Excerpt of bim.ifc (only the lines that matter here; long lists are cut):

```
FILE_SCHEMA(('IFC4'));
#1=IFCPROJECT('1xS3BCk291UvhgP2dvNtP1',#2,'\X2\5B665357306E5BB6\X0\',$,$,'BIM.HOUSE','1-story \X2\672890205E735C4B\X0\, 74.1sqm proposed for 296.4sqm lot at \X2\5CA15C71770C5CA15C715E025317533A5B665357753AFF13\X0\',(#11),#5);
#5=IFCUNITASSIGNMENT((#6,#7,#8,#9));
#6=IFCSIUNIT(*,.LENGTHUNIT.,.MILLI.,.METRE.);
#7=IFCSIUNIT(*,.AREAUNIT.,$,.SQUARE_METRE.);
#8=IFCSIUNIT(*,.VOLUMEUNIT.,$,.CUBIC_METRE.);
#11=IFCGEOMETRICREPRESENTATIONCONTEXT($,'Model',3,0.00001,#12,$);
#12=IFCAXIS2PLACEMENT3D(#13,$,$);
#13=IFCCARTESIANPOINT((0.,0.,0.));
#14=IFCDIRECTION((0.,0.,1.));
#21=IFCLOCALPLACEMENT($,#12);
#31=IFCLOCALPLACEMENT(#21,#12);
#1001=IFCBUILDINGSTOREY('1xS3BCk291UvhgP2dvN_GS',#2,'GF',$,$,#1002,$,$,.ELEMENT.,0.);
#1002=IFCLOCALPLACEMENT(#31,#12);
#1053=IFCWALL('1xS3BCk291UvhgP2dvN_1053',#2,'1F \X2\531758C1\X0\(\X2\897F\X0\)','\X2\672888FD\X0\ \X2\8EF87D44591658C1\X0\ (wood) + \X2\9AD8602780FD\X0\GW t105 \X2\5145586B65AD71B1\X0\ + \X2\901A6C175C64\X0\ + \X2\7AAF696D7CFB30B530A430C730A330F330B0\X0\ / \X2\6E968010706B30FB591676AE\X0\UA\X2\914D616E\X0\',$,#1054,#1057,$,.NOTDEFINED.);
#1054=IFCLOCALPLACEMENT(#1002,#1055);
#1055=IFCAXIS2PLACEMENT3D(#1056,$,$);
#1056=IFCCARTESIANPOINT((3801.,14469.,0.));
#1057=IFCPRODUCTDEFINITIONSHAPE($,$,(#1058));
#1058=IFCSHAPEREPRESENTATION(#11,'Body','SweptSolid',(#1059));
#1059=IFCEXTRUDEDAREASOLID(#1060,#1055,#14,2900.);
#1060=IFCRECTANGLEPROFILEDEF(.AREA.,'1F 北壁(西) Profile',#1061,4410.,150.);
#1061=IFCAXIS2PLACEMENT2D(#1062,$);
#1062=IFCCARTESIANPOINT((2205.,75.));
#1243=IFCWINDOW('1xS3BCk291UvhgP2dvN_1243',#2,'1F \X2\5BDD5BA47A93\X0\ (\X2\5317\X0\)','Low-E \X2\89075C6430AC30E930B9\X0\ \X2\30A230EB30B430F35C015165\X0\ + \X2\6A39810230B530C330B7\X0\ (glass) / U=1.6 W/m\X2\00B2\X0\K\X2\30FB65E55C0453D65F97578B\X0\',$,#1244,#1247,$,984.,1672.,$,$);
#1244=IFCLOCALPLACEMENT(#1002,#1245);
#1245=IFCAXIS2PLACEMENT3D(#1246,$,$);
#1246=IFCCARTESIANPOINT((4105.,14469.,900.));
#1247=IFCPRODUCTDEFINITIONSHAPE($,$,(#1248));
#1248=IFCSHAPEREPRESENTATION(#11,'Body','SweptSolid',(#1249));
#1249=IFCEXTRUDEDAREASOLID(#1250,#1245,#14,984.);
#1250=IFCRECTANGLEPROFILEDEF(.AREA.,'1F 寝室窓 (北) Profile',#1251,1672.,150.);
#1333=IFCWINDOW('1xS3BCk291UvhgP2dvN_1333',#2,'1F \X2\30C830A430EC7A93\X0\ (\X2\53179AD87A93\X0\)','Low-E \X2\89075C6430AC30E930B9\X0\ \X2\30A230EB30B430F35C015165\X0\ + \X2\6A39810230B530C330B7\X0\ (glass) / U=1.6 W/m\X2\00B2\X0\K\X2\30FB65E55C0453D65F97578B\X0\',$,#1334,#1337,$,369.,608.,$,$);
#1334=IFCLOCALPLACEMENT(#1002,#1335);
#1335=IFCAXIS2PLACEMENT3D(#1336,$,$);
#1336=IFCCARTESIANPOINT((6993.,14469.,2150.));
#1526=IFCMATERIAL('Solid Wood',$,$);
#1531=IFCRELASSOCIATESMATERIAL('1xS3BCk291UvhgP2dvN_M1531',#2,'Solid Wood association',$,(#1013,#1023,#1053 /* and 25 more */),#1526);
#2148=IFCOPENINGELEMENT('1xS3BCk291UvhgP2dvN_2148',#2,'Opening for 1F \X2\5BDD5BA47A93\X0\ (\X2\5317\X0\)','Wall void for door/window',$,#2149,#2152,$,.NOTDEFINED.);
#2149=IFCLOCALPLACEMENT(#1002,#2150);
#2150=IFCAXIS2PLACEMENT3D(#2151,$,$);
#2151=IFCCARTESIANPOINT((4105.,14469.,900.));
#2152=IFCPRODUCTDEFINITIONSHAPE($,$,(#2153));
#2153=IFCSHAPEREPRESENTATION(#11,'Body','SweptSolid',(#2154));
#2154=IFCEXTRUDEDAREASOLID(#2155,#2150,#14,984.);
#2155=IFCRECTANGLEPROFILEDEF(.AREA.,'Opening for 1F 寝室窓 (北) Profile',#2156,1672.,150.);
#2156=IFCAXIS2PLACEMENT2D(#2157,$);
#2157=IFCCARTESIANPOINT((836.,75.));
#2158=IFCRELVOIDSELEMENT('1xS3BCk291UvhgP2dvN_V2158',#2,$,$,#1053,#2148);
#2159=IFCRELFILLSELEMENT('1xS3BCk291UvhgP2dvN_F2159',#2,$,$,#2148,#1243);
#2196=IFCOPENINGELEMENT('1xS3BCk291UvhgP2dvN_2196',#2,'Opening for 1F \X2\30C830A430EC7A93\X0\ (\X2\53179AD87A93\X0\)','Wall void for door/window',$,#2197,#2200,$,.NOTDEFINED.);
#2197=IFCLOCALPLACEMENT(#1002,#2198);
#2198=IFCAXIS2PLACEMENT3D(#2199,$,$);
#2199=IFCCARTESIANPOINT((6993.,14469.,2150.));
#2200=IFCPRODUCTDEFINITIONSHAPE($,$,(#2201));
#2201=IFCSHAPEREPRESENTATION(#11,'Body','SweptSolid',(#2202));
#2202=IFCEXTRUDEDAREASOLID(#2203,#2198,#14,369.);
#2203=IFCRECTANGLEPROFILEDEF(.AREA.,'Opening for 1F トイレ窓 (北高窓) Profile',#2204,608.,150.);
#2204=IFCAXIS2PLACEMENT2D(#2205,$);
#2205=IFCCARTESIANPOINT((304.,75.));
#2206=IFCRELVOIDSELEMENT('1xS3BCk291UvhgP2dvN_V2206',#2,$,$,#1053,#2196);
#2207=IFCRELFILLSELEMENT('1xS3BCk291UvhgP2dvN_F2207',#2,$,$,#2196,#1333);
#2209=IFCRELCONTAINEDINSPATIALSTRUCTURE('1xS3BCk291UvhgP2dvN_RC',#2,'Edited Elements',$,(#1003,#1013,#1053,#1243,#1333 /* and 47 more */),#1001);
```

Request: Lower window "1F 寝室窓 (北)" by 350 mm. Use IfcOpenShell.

```python
import numpy as np
import ifcopenshell
import ifcopenshell.api.geometry
import ifcopenshell.util.placement
import ifcopenshell.util.unit

model = ifcopenshell.open("bim.ifc")
unit_scale = ifcopenshell.util.unit.calculate_unit_scale(model)

window = model.by_id(1243)
opening = window.FillsVoids[0].RelatingOpeningElement
dz = -0.35 / unit_scale

shift = np.array([0.0, 0.0, dz])
# The window is not placed relative to its opening, so move both.
for product in (opening, window):
    matrix = ifcopenshell.util.placement.get_local_placement(product.ObjectPlacement)
    matrix[:3, 3] += shift
    ifcopenshell.api.geometry.edit_object_placement(model, product=product, matrix=matrix, is_si=False)

print(f"moved by {dz * unit_scale:+.3f} m")

model.write("bim_edited.ifc")
```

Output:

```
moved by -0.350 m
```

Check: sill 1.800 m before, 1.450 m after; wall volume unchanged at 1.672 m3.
